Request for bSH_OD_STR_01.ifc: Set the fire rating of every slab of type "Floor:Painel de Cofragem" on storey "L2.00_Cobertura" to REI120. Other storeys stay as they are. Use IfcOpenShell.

First a look at what the model holds.

```python
import ifcopenshell
import ifcopenshell.util.element

model = ifcopenshell.open("bSH_OD_STR_01.ifc")
print(model.schema)
storey = next(s for s in model.by_type("IfcBuildingStorey") if s.Name == "L2.00_Cobertura")
slabs = [e for e in ifcopenshell.util.element.get_decomposition(storey) if e.is_a("IfcSlab")]
seen = {}
for e in slabs:
    element_type = ifcopenshell.util.element.get_type(e)
    key = (element_type.Name if element_type != e and element_type else None, ifcopenshell.util.element.get_pset(e, "Pset_SlabCommon", "FireRating"))
    seen[key] = seen.get(key, 0) + 1
for (name, value), count in sorted(seen.items(), key=str):
    print(count, "x", name, "|", value)
```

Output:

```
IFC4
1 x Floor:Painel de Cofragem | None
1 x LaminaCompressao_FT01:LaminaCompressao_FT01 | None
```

```python
import ifcopenshell
import ifcopenshell.api.pset
import ifcopenshell.util.element

model = ifcopenshell.open("bSH_OD_STR_01.ifc")

storey = next(s for s in model.by_type("IfcBuildingStorey") if s.Name == "L2.00_Cobertura")
slabs = [e for e in ifcopenshell.util.element.get_decomposition(storey) if e.is_a("IfcSlab")]

count = 0
for e in slabs:
    element_type = ifcopenshell.util.element.get_type(e)
    if element_type in (None, e) or element_type.Name != "Floor:Painel de Cofragem":
        continue
    # add_pset returns the element's existing set when there is one.
    pset = ifcopenshell.api.pset.add_pset(model, product=e, name="Pset_SlabCommon")
    ifcopenshell.api.pset.edit_pset(model, pset=pset, properties={"FireRating": "REI120"})
    count += 1

print(count, "slabs updated")

model.write("bSH_OD_STR_01_edited.ifc")
```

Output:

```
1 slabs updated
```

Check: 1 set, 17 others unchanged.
